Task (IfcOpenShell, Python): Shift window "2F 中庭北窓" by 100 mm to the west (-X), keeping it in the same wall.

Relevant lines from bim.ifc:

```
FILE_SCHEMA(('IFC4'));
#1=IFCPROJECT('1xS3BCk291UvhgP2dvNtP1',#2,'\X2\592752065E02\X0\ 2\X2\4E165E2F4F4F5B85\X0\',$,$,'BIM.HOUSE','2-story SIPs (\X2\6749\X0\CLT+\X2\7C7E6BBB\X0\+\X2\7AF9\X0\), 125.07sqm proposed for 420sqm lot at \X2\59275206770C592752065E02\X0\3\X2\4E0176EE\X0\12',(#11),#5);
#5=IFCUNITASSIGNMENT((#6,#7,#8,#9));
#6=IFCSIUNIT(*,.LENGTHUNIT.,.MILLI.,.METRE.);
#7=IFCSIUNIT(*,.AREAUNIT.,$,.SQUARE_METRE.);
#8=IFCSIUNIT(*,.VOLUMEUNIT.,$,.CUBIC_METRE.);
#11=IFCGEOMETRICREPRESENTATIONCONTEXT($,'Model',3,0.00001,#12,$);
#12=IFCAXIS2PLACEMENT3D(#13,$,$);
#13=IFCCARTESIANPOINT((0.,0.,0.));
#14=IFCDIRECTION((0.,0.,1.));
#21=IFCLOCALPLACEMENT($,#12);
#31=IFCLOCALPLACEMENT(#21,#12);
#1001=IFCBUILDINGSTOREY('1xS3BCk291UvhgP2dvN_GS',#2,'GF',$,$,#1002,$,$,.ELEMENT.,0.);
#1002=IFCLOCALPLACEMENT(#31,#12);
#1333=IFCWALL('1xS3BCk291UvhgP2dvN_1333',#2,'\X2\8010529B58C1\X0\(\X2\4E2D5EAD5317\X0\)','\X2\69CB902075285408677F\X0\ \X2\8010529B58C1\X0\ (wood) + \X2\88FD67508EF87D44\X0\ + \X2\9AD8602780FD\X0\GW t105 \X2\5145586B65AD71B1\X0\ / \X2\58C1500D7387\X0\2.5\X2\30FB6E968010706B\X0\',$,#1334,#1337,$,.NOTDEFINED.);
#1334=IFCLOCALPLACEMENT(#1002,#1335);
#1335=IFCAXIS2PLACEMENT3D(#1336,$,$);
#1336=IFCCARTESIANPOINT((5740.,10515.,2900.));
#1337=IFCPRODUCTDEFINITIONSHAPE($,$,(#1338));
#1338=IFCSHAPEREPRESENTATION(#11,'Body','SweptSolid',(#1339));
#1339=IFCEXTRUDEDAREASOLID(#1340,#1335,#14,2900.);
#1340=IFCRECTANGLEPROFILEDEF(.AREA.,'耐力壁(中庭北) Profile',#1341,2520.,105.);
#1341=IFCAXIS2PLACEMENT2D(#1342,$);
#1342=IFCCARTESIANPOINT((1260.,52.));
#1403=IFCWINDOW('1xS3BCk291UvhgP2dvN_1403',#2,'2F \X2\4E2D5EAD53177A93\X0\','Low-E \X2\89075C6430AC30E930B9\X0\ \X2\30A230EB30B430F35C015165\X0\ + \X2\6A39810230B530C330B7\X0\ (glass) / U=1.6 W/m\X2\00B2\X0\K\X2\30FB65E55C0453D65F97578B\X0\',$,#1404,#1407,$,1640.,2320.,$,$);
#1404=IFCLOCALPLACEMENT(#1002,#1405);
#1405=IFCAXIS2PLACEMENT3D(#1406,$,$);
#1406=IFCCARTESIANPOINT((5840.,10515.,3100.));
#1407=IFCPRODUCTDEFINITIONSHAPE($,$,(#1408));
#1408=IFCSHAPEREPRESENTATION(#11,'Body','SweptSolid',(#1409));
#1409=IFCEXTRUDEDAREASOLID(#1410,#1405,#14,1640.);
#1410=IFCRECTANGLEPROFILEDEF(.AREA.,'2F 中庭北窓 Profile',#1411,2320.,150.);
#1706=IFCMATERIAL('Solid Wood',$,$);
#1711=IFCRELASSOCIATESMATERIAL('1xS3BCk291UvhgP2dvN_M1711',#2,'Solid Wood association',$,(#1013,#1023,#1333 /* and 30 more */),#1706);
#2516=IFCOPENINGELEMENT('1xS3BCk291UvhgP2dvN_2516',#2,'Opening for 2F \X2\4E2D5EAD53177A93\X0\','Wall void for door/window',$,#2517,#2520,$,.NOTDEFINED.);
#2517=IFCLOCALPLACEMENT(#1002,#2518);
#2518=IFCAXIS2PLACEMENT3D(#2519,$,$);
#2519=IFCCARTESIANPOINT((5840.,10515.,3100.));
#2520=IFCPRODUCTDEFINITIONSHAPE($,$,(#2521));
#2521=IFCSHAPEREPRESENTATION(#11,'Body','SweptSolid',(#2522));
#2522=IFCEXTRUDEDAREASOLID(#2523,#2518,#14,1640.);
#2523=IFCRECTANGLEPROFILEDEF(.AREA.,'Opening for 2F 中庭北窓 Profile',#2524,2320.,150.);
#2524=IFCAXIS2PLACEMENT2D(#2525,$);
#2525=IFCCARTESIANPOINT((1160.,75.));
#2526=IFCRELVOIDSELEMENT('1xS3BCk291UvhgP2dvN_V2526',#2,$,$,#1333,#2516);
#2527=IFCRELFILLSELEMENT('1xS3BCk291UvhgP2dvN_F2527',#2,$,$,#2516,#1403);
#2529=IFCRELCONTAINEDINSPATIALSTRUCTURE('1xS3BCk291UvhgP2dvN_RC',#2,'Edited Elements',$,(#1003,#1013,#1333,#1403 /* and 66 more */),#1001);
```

```python
import ifcopenshell
import ifcopenshell.api.geometry
import ifcopenshell.util.placement

model = ifcopenshell.open("bim.ifc")

window = model.by_id(1403)
opening = window.FillsVoids[0].RelatingOpeningElement
wall = opening.VoidsElements[0].RelatingBuildingElement

wall_matrix = ifcopenshell.util.placement.get_local_placement(wall.ObjectPlacement)
shift = wall_matrix[:3, 0] * -100.0
before = ifcopenshell.util.placement.get_local_placement(window.ObjectPlacement)[:3, 3].copy()

# The window is not placed relative to its opening, so move both.
for product in (opening, window):
    matrix = ifcopenshell.util.placement.get_local_placement(product.ObjectPlacement)
    matrix[:3, 3] += shift
    ifcopenshell.api.geometry.edit_object_placement(model, product=product, matrix=matrix, is_si=False)

after = ifcopenshell.util.placement.get_local_placement(window.ObjectPlacement)[:3, 3]
print("window moved by", (after - before).round(3) + 0.0)

model.write("bim_edited.ifc")
```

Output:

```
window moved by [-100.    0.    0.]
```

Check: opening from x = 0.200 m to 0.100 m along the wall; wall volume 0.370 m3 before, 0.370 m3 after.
